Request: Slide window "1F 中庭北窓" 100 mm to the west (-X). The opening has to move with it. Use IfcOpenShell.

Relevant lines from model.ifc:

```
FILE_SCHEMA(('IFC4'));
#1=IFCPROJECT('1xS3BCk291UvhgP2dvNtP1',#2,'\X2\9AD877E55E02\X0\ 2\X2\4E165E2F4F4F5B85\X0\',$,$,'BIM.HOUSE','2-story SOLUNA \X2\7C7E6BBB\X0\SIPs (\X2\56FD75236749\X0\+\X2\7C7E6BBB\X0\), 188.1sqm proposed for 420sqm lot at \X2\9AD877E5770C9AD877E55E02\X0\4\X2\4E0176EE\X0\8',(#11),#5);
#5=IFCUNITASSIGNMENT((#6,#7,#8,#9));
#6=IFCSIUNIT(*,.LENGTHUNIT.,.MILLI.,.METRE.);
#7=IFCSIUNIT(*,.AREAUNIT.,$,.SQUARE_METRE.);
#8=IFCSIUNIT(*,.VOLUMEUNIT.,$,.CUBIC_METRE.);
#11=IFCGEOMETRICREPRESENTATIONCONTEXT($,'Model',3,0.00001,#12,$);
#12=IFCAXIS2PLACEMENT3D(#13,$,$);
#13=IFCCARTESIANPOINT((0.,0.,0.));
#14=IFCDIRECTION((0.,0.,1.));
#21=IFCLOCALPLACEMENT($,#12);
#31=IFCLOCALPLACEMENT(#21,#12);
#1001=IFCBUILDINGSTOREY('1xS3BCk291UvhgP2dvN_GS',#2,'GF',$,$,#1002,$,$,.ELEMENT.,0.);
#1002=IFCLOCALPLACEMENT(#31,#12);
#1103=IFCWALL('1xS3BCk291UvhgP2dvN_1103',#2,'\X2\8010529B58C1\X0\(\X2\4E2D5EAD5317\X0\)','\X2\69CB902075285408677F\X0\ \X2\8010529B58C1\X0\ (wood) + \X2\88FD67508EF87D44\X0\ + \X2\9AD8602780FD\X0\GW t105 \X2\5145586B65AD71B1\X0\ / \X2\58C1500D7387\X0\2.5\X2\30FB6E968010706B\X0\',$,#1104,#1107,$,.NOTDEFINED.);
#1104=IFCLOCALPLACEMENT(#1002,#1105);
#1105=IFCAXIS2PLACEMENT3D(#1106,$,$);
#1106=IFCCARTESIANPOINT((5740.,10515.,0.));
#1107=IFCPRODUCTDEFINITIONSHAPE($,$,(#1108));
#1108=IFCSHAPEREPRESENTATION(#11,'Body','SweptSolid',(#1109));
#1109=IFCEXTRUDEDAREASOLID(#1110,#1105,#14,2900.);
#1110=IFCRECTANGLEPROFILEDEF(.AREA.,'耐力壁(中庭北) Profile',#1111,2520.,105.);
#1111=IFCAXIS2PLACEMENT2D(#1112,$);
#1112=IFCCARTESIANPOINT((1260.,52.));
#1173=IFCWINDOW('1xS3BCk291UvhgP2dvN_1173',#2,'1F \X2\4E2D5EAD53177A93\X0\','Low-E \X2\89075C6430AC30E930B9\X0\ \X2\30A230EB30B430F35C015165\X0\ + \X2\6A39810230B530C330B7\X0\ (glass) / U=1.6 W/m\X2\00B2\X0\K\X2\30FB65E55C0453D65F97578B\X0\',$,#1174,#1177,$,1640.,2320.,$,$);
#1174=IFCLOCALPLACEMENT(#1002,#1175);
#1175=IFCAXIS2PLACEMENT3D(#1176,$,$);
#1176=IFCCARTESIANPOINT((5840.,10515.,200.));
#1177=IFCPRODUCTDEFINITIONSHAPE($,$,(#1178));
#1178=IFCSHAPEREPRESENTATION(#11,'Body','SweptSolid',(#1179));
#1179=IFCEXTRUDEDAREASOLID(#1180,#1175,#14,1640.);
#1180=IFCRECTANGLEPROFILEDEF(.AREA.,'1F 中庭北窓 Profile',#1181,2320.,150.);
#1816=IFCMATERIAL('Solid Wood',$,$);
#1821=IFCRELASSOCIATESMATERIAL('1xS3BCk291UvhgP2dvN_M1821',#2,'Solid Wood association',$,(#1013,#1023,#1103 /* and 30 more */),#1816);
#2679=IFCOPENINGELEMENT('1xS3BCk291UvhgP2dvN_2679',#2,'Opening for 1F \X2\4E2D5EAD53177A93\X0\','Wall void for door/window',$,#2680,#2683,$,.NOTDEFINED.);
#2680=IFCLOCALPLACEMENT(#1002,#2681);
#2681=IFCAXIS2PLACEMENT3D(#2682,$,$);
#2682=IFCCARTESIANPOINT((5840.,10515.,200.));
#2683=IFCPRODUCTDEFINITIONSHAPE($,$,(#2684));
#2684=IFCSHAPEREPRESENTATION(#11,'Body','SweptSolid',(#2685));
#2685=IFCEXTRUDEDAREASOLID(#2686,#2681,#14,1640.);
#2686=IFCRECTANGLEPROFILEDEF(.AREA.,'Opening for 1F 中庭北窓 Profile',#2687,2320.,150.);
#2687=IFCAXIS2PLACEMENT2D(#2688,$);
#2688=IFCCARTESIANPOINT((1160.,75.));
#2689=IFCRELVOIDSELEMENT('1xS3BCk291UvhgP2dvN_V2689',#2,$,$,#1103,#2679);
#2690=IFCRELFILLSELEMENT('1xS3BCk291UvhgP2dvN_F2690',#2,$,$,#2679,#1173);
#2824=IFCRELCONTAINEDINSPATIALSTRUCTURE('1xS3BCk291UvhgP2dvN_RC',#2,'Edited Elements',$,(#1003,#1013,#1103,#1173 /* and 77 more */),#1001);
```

```python
import ifcopenshell
import ifcopenshell.api.geometry
import ifcopenshell.util.placement

model = ifcopenshell.open("model.ifc")

window = model.by_id(1173)
opening = window.FillsVoids[0].RelatingOpeningElement
wall = opening.VoidsElements[0].RelatingBuildingElement

wall_matrix = ifcopenshell.util.placement.get_local_placement(wall.ObjectPlacement)
shift = wall_matrix[:3, 0] * -100.0
before = ifcopenshell.util.placement.get_local_placement(window.ObjectPlacement)[:3, 3].copy()

# The window is not placed relative to its opening, so move both.
for product in (opening, window):
    matrix = ifcopenshell.util.placement.get_local_placement(product.ObjectPlacement)
    matrix[:3, 3] += shift
    ifcopenshell.api.geometry.edit_object_placement(model, product=product, matrix=matrix, is_si=False)

after = ifcopenshell.util.placement.get_local_placement(window.ObjectPlacement)[:3, 3]
print("window moved by", (after - before).round(3) + 0.0)

model.write("model_edited.ifc")
```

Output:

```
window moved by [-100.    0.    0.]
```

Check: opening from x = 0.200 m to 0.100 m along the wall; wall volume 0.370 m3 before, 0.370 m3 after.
